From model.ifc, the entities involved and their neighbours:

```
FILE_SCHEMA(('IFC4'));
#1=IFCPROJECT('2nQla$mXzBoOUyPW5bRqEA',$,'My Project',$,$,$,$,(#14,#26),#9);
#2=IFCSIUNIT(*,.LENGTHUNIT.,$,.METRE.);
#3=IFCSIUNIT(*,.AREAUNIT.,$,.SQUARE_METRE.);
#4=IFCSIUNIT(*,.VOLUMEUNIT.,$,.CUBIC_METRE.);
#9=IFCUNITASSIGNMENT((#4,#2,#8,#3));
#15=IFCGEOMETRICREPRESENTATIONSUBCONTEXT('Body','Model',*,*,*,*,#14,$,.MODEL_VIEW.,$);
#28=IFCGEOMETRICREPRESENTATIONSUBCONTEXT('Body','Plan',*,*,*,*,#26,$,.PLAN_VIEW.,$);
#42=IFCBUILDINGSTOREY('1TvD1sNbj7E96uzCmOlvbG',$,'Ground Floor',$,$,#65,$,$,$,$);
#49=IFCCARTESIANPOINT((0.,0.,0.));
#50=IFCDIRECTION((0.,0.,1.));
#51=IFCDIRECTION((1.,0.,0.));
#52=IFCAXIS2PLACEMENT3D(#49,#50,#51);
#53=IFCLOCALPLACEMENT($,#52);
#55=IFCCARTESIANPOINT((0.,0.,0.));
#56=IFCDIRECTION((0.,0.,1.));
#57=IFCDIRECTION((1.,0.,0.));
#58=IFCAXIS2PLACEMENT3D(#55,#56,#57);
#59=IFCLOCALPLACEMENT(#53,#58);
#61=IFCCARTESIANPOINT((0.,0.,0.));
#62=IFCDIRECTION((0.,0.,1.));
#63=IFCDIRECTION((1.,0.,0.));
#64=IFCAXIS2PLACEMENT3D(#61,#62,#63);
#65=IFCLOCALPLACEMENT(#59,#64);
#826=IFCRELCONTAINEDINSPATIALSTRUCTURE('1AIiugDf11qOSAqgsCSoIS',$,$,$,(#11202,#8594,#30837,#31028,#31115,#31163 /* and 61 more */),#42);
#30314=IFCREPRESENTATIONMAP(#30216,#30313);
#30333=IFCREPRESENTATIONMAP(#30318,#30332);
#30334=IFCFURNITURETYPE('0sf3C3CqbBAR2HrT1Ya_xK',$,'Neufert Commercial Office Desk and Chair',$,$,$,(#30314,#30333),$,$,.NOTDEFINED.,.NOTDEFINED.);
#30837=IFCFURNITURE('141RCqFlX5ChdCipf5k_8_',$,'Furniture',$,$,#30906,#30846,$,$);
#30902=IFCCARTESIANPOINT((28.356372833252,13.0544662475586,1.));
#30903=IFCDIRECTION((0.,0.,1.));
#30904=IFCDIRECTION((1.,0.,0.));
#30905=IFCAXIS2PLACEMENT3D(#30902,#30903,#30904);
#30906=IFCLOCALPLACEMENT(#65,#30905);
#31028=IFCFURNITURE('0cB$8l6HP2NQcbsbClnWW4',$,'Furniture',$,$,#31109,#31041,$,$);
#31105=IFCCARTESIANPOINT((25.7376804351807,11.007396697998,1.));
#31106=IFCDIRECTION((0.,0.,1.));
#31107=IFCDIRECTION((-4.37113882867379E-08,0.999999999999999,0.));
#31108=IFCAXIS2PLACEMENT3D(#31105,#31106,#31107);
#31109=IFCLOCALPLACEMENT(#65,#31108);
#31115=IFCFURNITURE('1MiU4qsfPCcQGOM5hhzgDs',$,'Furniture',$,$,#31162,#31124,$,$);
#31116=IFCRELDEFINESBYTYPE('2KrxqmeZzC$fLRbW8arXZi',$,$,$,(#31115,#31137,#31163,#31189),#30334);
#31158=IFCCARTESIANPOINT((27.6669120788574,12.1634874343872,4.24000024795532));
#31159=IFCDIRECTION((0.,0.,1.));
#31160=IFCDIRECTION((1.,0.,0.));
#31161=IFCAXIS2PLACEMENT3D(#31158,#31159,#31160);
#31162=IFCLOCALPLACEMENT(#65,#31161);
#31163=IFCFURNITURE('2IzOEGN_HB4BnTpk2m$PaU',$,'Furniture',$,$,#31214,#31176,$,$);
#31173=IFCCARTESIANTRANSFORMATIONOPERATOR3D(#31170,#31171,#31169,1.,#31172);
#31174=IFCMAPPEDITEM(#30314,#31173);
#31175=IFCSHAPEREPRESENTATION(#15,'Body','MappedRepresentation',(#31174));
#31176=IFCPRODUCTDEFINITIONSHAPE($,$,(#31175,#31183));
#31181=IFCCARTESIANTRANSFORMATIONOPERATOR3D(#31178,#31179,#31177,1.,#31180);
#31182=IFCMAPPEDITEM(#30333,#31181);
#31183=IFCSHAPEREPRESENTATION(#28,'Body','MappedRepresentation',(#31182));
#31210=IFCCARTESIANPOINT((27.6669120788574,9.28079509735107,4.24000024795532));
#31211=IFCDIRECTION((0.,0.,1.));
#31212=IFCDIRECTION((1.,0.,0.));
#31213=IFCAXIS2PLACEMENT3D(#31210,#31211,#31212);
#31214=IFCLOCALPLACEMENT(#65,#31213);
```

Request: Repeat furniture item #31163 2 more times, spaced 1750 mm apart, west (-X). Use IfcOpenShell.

```python
import numpy as np
import ifcopenshell
import ifcopenshell.api.geometry
import ifcopenshell.api.root
import ifcopenshell.util.element
import ifcopenshell.util.placement

model = ifcopenshell.open("model.ifc")

source = model.by_guid("2IzOEGN_HB4BnTpk2m$PaU")
base = ifcopenshell.util.placement.get_local_placement(source.ObjectPlacement)
step = np.array([-1.0, 0.0, 0.0]) * 1.75

for i in range(1, 3):
    copy = ifcopenshell.api.root.copy_class(model, product=source)
    copy.Representation = ifcopenshell.util.element.copy_deep(
        model, source.Representation, exclude=["IfcGeometricRepresentationContext", "IfcRepresentationMap"]
    )
    matrix = base.copy()
    matrix[:3, 3] += i * step
    print("added at", matrix[:3, 3].round(3) + 0.0)
    ifcopenshell.api.geometry.edit_object_placement(model, product=copy, matrix=matrix, is_si=False)

model.write("model-out.ifc")
```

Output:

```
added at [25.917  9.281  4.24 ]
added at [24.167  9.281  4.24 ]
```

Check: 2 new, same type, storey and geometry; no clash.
